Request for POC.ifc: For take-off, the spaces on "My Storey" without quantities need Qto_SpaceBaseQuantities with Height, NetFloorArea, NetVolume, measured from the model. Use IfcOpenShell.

First a look at what the model holds.

```python
import ifcopenshell
import ifcopenshell.util.element
import ifcopenshell.util.unit

model = ifcopenshell.open("POC.ifc")
print(model.schema)
for unit_type in ("LENGTHUNIT", "AREAUNIT", "VOLUMEUNIT"):
    print(unit_type, ifcopenshell.util.unit.calculate_unit_scale(model, unit_type))
storey = next(s for s in model.by_type("IfcBuildingStorey") if s.Name == "My Storey")
spaces = [e for e in ifcopenshell.util.element.get_decomposition(storey) if e.is_a("IfcSpace")]
for e in sorted(spaces, key=lambda e: e.id()):
    print(e.id(), e.is_a(), e.Name, list(ifcopenshell.util.element.get_psets(e, qtos_only=True)), sep=" | ")
```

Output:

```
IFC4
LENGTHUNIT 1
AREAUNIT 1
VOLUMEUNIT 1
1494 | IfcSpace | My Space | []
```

```python
import ifcopenshell
import ifcopenshell.api.pset
import ifcopenshell.geom
import ifcopenshell.util.element
import ifcopenshell.util.shape
import ifcopenshell.util.unit

model = ifcopenshell.open("POC.ifc")
unit_scale = ifcopenshell.util.unit.calculate_unit_scale(model)
area_scale = ifcopenshell.util.unit.calculate_unit_scale(model, "AREAUNIT")
volume_scale = ifcopenshell.util.unit.calculate_unit_scale(model, "VOLUMEUNIT")
settings = ifcopenshell.geom.settings()

storey = next(s for s in model.by_type("IfcBuildingStorey") if s.Name == "My Storey")
spaces = [e for e in ifcopenshell.util.element.get_decomposition(storey) if e.is_a("IfcSpace")]

for e in sorted(spaces, key=lambda e: e.id()):
    if ifcopenshell.util.element.get_psets(e, qtos_only=True, should_inherit=False):
        continue
    # Geometry comes back in metres, in the element's own axes.
    shape = ifcopenshell.geom.create_shape(settings, e)
    values = {
        "Height": ifcopenshell.util.shape.get_z(shape.geometry) / unit_scale,
        "NetFloorArea": ifcopenshell.util.shape.get_footprint_area(shape.geometry) / area_scale,
        "NetVolume": ifcopenshell.util.shape.get_volume(shape.geometry) / volume_scale,
    }
    qto = ifcopenshell.api.pset.add_qto(model, product=e, name="Qto_SpaceBaseQuantities")
    ifcopenshell.api.pset.edit_qto(model, qto=qto, properties=values)
    print(e.id(), {k: round(v, 3) for k, v in values.items()})

model.write("POC-out.ifc")
```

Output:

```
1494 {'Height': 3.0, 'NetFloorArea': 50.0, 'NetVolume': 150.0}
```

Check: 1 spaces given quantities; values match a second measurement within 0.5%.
